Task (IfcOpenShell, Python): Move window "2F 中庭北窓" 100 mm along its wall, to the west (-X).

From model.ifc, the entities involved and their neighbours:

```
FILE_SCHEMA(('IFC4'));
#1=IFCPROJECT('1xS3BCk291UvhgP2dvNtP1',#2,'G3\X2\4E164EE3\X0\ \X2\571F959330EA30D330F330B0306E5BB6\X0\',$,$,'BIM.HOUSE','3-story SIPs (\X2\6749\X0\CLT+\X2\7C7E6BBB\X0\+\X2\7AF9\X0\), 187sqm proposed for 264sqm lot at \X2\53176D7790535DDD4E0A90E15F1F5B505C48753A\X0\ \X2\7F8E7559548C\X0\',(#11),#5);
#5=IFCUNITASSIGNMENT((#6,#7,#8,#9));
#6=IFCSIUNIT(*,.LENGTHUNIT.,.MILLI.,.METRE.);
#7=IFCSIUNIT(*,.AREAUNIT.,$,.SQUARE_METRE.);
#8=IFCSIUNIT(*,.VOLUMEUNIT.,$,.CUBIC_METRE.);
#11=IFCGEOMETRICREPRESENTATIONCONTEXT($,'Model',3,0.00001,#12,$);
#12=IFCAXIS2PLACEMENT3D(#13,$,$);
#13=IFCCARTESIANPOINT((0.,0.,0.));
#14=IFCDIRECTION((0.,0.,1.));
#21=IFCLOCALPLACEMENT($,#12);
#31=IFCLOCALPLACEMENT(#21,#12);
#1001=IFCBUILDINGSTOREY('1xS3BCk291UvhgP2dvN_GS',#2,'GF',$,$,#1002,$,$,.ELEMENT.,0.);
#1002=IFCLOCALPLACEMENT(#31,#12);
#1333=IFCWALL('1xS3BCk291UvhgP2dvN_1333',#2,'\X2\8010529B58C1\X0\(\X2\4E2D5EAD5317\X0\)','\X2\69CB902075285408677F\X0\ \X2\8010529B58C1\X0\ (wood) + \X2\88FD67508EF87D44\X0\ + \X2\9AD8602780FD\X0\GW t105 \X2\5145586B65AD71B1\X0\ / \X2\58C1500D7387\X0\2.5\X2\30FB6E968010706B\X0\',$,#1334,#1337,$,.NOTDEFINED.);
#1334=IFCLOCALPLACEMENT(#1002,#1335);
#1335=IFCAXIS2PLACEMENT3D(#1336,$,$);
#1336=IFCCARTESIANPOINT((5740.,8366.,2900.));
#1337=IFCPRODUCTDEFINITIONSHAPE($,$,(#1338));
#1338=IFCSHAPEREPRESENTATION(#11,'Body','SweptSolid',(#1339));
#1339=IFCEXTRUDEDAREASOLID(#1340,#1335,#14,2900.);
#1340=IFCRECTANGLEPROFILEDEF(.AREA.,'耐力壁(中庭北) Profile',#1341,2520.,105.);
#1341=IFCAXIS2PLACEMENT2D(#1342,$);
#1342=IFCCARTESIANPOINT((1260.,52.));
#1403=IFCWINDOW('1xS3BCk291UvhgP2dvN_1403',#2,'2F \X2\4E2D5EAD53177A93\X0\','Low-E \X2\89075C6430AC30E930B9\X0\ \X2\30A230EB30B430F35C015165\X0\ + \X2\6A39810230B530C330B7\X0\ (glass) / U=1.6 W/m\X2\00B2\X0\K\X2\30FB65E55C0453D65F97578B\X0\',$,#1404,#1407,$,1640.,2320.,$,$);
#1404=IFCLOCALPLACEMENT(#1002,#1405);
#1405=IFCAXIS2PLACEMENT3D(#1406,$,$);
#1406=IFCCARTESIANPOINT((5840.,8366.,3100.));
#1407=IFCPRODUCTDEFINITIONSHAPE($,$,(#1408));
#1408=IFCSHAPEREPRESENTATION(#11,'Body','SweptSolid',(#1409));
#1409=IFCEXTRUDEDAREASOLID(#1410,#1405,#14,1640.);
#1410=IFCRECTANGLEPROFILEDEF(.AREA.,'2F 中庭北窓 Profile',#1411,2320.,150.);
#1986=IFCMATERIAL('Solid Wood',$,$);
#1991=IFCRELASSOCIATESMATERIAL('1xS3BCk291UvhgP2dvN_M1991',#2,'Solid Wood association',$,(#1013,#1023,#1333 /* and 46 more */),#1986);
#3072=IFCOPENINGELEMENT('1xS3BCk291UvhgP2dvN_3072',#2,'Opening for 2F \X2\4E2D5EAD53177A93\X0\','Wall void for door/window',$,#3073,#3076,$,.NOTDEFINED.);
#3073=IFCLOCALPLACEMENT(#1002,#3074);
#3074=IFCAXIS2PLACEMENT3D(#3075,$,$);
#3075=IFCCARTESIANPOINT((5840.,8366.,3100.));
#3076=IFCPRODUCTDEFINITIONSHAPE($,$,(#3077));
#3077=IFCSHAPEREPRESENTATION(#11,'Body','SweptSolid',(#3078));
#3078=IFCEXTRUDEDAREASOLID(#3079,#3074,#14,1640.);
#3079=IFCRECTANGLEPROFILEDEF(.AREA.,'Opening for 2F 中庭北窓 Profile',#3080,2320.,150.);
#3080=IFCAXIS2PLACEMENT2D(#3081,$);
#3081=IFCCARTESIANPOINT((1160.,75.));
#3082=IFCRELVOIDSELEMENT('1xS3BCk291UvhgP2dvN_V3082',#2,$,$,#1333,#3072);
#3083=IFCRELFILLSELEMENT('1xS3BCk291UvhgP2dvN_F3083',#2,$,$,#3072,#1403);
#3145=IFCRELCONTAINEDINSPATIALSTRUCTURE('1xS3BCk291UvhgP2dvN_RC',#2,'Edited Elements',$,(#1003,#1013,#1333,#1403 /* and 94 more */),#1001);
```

```python
import ifcopenshell
import ifcopenshell.api.geometry
import ifcopenshell.util.placement

model = ifcopenshell.open("model.ifc")

window = model.by_guid("1xS3BCk291UvhgP2dvN_1403")
opening = window.FillsVoids[0].RelatingOpeningElement
wall = opening.VoidsElements[0].RelatingBuildingElement

wall_matrix = ifcopenshell.util.placement.get_local_placement(wall.ObjectPlacement)
shift = wall_matrix[:3, 0] * -100.0
before = ifcopenshell.util.placement.get_local_placement(window.ObjectPlacement)[:3, 3].copy()

# The window is not placed relative to its opening, so move both.
for product in (opening, window):
    matrix = ifcopenshell.util.placement.get_local_placement(product.ObjectPlacement)
    matrix[:3, 3] += shift
    ifcopenshell.api.geometry.edit_object_placement(model, product=product, matrix=matrix, is_si=False)

after = ifcopenshell.util.placement.get_local_placement(window.ObjectPlacement)[:3, 3]
print("window moved by", (after - before).round(3) + 0.0)

model.write("model_v2.ifc")
```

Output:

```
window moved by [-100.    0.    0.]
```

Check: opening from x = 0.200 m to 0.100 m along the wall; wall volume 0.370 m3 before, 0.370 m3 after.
